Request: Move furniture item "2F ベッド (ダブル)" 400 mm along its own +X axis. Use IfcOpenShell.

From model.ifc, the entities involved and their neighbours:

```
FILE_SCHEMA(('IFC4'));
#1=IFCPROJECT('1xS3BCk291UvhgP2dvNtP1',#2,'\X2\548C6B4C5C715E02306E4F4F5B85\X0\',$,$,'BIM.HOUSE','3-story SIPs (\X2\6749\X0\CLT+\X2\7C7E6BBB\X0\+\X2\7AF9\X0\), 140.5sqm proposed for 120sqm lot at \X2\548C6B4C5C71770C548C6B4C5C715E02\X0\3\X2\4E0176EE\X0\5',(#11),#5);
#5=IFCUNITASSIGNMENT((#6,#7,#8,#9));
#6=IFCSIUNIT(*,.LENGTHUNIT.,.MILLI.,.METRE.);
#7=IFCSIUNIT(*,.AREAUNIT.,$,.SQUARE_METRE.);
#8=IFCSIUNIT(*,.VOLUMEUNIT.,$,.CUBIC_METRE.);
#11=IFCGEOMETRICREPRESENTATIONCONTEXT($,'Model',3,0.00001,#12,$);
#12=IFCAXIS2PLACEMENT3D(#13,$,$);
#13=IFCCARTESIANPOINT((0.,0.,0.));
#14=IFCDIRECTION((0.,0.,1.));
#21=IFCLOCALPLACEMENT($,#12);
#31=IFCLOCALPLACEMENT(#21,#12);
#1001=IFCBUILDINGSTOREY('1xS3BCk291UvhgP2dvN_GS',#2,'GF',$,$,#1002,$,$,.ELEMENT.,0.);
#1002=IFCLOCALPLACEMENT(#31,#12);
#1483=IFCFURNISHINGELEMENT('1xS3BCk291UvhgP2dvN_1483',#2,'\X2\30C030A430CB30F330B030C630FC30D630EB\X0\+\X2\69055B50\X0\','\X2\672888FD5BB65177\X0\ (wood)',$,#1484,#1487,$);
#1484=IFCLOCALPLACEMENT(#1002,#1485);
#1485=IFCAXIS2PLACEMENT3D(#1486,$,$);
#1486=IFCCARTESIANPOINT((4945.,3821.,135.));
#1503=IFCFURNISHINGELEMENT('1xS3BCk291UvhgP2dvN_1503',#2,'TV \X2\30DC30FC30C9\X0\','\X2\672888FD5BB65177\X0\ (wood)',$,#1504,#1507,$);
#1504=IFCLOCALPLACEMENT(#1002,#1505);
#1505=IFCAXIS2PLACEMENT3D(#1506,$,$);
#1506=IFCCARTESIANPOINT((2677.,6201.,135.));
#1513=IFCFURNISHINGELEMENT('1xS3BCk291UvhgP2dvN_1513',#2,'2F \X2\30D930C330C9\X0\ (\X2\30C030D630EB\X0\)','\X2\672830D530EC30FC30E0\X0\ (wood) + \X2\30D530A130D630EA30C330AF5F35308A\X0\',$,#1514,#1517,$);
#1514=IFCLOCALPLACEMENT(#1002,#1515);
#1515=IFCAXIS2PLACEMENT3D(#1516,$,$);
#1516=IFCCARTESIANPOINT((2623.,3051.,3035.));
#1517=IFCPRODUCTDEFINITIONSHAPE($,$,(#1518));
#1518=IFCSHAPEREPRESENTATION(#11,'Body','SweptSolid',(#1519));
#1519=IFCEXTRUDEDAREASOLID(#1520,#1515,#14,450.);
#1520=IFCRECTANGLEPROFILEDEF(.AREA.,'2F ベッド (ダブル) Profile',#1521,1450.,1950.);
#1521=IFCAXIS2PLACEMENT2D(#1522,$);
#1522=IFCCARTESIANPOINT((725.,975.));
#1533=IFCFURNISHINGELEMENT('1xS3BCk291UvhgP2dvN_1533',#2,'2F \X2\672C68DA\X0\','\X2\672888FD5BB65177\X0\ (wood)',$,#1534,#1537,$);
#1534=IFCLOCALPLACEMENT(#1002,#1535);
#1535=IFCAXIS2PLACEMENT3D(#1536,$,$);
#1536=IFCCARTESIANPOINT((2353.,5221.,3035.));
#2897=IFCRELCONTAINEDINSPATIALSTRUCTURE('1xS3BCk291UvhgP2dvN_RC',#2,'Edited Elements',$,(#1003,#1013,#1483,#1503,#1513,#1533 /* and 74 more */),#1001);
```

```python
import ifcopenshell
import ifcopenshell.api.geometry
import ifcopenshell.util.placement
import ifcopenshell.util.unit

model = ifcopenshell.open("model.ifc")
unit_scale = ifcopenshell.util.unit.calculate_unit_scale(model)

item = model.by_id(1513)
matrix = ifcopenshell.util.placement.get_local_placement(item.ObjectPlacement)
matrix[:3, 3] += matrix[:3, 0] * 0.4 / unit_scale
ifcopenshell.api.geometry.edit_object_placement(model, product=item, matrix=matrix, is_si=False)

print(ifcopenshell.util.placement.get_local_placement(item.ObjectPlacement).round(3) + 0.0)

model.write("model_updated.ifc")
```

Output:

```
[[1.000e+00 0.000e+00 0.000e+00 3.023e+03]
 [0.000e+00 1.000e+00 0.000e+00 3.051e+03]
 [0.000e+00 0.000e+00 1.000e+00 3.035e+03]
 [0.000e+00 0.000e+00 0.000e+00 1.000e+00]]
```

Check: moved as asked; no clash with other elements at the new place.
